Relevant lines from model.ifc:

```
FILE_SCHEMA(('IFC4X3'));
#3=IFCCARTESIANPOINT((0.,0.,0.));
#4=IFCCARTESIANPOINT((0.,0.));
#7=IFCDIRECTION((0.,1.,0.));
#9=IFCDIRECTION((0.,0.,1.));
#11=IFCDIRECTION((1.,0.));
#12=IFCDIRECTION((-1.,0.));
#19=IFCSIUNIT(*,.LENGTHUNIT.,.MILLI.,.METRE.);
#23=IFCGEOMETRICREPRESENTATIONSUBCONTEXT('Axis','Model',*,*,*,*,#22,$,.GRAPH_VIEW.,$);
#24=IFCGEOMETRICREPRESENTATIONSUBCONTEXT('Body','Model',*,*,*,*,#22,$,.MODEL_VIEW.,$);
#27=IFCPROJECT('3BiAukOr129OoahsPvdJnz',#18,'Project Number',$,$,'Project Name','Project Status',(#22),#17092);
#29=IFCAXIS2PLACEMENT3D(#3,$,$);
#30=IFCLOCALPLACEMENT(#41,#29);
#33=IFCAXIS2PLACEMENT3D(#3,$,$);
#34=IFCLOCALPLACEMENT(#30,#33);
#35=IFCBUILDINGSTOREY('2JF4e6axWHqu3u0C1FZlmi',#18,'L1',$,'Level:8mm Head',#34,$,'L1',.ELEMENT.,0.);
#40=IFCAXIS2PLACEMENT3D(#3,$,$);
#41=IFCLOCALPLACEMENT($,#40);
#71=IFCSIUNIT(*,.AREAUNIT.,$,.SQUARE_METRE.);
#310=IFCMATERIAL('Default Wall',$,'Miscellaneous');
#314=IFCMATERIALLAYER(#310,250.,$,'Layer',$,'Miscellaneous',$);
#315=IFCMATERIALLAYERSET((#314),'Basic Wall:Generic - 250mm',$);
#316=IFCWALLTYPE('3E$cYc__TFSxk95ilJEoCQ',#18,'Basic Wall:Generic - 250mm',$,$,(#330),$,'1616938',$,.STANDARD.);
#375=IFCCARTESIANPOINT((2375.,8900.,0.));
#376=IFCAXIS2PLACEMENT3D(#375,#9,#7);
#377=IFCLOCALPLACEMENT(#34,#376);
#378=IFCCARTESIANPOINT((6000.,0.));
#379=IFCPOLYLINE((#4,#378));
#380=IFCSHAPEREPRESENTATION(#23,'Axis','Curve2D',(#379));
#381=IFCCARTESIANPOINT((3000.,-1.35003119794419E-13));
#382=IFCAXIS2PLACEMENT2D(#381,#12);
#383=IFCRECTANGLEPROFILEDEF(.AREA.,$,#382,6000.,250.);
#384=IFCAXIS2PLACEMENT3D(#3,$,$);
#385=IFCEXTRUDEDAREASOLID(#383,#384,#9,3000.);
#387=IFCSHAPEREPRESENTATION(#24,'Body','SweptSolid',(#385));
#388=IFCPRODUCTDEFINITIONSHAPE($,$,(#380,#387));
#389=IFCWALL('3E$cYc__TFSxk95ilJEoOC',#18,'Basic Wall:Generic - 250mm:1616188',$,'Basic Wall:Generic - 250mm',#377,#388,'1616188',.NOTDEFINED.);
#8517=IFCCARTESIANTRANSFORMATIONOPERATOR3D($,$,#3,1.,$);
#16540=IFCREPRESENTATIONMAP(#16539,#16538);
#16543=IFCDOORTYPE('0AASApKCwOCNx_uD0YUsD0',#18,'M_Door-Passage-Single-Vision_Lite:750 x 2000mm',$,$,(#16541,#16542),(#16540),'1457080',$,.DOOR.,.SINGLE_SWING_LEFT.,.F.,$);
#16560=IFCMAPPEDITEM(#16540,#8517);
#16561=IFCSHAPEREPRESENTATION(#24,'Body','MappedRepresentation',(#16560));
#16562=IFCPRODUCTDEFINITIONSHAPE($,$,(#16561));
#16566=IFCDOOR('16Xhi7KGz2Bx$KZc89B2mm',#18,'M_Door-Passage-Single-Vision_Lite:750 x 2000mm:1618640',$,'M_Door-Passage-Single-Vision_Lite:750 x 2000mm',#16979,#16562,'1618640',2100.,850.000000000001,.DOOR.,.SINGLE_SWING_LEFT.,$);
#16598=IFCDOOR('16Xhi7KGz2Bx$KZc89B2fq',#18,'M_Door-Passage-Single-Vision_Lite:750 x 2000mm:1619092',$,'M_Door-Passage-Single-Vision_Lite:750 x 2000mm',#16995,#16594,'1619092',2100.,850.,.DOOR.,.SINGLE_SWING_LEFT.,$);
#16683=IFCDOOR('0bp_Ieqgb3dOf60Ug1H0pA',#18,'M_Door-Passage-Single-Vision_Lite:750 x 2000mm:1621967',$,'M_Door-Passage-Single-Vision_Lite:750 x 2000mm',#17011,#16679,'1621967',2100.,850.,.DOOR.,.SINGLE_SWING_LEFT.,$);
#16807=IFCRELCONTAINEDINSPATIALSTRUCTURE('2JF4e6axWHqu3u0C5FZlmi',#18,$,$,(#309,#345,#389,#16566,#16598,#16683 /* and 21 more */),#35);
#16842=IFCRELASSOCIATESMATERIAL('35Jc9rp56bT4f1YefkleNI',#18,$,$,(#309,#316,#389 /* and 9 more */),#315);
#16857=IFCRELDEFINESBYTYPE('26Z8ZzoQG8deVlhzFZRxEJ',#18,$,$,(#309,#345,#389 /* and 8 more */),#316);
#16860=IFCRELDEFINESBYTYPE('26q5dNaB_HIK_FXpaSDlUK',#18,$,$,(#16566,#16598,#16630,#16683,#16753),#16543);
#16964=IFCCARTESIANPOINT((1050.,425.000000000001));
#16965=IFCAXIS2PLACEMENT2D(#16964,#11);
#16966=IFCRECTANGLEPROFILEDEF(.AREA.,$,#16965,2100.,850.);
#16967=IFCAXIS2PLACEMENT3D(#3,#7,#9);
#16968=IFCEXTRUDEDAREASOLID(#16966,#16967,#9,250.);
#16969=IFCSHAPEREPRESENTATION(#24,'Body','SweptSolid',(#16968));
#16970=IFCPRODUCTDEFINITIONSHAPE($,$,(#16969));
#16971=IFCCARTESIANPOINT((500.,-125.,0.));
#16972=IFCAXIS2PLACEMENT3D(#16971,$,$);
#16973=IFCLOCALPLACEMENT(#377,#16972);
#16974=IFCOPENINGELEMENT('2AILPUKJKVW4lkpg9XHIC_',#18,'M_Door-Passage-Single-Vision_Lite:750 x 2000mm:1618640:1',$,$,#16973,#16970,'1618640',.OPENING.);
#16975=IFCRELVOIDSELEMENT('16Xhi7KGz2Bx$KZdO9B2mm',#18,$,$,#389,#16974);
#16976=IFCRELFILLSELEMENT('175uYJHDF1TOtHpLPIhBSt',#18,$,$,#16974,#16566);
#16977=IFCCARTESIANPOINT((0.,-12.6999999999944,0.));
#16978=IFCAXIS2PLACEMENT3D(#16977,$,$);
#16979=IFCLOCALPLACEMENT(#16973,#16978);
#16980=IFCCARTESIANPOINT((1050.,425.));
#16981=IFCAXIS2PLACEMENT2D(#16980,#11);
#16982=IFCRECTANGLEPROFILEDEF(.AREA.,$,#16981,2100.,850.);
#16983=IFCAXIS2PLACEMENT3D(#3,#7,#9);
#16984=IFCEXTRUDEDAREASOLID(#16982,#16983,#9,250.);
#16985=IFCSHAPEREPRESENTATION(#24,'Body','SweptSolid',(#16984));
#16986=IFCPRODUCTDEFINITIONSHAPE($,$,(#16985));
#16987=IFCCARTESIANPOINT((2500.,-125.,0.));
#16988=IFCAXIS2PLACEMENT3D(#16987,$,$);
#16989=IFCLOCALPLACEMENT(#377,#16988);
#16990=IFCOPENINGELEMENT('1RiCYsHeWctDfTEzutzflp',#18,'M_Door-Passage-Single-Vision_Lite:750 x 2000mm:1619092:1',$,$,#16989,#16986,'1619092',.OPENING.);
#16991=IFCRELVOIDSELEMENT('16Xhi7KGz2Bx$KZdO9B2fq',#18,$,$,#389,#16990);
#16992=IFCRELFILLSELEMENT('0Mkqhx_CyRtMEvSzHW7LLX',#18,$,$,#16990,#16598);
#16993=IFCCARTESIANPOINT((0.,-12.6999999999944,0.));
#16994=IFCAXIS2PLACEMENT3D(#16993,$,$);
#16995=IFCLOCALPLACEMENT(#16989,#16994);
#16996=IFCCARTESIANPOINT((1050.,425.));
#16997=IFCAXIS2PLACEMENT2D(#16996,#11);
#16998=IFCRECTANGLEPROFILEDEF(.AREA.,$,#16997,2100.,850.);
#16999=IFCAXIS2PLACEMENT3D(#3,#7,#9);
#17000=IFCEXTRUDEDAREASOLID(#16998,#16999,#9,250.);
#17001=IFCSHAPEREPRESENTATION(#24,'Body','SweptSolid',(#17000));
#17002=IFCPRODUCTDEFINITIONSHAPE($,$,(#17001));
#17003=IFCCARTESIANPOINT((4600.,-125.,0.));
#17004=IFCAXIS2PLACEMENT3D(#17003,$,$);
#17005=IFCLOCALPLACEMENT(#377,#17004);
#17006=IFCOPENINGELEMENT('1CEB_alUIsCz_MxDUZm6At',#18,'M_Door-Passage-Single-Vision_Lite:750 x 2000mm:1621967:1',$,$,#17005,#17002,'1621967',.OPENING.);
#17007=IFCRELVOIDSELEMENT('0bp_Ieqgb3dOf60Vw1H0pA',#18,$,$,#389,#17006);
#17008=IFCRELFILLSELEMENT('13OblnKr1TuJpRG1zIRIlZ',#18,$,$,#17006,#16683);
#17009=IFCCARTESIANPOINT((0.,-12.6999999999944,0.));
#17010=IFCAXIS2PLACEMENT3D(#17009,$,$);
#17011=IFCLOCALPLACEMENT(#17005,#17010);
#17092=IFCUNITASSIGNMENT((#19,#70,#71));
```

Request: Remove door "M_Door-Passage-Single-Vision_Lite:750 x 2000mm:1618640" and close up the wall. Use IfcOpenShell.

```python
import ifcopenshell
import ifcopenshell.api.feature
import ifcopenshell.api.root
import ifcopenshell.geom
import ifcopenshell.util.shape

model = ifcopenshell.open("model.ifc")
settings = ifcopenshell.geom.settings()


def volume(element):
    """Net volume in cubic metres, openings subtracted."""
    shape = ifcopenshell.geom.create_shape(settings, element)
    return ifcopenshell.util.shape.get_volume(shape.geometry)


door = model.by_guid("16Xhi7KGz2Bx$KZc89B2mm")
opening = door.FillsVoids[0].RelatingOpeningElement
wall = opening.VoidsElements[0].RelatingBuildingElement
before = volume(wall)

ifcopenshell.api.root.remove_product(model, product=door)
ifcopenshell.api.feature.remove_feature(model, feature=opening)

after = volume(wall)

print(f"wall volume {before:.3f} -> {after:.3f} m3")

model.write("model_edited.ifc")
```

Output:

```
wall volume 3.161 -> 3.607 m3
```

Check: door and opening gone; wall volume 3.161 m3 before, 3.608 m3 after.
